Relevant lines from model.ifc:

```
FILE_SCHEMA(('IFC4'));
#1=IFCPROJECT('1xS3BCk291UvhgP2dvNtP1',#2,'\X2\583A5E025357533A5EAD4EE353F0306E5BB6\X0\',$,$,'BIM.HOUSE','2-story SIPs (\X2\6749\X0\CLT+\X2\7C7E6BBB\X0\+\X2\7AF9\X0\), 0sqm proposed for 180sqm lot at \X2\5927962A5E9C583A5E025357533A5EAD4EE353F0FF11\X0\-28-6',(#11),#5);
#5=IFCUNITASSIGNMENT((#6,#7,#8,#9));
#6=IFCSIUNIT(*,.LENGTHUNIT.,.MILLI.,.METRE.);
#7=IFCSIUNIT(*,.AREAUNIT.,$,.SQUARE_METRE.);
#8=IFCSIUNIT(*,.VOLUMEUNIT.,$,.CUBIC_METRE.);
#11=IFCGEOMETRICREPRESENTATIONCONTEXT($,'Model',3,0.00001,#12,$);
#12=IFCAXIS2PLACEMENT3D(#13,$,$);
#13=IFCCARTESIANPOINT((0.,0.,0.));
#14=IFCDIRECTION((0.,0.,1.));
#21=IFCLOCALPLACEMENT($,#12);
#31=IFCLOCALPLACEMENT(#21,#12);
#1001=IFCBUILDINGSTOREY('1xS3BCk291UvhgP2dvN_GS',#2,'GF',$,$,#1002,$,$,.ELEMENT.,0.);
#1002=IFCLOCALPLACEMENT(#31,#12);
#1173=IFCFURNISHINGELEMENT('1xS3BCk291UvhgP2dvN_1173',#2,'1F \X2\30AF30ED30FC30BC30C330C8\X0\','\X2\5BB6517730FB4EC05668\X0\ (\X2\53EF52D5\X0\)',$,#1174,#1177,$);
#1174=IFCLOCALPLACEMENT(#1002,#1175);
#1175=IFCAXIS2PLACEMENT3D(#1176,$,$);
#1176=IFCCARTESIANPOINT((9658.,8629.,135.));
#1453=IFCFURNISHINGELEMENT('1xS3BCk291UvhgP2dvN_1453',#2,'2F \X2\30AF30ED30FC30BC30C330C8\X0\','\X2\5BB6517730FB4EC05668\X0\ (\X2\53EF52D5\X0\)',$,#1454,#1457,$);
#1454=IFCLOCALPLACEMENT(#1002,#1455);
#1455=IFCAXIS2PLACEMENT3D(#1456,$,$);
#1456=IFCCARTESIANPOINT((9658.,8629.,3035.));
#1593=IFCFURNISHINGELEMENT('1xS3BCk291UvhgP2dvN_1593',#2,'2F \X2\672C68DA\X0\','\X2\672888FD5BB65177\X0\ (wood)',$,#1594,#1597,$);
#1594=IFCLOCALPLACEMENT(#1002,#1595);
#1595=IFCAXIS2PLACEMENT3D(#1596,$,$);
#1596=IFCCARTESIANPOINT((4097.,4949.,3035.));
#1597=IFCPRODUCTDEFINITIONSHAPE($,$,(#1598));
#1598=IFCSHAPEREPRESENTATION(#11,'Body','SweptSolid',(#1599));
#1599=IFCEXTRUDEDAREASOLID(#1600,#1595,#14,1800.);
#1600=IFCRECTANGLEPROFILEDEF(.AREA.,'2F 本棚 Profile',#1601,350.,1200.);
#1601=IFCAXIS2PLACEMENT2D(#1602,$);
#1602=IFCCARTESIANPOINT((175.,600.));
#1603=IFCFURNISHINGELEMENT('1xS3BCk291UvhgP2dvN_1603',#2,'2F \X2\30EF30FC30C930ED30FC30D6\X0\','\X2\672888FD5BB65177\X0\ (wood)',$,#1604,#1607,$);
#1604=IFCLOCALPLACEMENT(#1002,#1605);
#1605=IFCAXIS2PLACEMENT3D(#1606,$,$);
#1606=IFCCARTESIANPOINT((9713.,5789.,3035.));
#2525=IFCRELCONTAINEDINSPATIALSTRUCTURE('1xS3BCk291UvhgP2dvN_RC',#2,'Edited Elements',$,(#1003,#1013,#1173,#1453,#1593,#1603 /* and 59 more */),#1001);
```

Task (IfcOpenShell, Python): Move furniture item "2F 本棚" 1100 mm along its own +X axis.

```python
import ifcopenshell
import ifcopenshell.api.geometry
import ifcopenshell.util.placement

model = ifcopenshell.open("model.ifc")

item = model.by_guid("1xS3BCk291UvhgP2dvN_1593")
matrix = ifcopenshell.util.placement.get_local_placement(item.ObjectPlacement)
matrix[:3, 3] += matrix[:3, 0] * 1100.0
ifcopenshell.api.geometry.edit_object_placement(model, product=item, matrix=matrix, is_si=False)

print(ifcopenshell.util.placement.get_local_placement(item.ObjectPlacement).round(3) + 0.0)

model.write("model_updated.ifc")
```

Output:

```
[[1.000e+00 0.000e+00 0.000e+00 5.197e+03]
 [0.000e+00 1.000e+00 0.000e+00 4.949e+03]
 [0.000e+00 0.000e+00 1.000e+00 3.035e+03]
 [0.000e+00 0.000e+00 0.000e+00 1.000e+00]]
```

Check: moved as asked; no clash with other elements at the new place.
